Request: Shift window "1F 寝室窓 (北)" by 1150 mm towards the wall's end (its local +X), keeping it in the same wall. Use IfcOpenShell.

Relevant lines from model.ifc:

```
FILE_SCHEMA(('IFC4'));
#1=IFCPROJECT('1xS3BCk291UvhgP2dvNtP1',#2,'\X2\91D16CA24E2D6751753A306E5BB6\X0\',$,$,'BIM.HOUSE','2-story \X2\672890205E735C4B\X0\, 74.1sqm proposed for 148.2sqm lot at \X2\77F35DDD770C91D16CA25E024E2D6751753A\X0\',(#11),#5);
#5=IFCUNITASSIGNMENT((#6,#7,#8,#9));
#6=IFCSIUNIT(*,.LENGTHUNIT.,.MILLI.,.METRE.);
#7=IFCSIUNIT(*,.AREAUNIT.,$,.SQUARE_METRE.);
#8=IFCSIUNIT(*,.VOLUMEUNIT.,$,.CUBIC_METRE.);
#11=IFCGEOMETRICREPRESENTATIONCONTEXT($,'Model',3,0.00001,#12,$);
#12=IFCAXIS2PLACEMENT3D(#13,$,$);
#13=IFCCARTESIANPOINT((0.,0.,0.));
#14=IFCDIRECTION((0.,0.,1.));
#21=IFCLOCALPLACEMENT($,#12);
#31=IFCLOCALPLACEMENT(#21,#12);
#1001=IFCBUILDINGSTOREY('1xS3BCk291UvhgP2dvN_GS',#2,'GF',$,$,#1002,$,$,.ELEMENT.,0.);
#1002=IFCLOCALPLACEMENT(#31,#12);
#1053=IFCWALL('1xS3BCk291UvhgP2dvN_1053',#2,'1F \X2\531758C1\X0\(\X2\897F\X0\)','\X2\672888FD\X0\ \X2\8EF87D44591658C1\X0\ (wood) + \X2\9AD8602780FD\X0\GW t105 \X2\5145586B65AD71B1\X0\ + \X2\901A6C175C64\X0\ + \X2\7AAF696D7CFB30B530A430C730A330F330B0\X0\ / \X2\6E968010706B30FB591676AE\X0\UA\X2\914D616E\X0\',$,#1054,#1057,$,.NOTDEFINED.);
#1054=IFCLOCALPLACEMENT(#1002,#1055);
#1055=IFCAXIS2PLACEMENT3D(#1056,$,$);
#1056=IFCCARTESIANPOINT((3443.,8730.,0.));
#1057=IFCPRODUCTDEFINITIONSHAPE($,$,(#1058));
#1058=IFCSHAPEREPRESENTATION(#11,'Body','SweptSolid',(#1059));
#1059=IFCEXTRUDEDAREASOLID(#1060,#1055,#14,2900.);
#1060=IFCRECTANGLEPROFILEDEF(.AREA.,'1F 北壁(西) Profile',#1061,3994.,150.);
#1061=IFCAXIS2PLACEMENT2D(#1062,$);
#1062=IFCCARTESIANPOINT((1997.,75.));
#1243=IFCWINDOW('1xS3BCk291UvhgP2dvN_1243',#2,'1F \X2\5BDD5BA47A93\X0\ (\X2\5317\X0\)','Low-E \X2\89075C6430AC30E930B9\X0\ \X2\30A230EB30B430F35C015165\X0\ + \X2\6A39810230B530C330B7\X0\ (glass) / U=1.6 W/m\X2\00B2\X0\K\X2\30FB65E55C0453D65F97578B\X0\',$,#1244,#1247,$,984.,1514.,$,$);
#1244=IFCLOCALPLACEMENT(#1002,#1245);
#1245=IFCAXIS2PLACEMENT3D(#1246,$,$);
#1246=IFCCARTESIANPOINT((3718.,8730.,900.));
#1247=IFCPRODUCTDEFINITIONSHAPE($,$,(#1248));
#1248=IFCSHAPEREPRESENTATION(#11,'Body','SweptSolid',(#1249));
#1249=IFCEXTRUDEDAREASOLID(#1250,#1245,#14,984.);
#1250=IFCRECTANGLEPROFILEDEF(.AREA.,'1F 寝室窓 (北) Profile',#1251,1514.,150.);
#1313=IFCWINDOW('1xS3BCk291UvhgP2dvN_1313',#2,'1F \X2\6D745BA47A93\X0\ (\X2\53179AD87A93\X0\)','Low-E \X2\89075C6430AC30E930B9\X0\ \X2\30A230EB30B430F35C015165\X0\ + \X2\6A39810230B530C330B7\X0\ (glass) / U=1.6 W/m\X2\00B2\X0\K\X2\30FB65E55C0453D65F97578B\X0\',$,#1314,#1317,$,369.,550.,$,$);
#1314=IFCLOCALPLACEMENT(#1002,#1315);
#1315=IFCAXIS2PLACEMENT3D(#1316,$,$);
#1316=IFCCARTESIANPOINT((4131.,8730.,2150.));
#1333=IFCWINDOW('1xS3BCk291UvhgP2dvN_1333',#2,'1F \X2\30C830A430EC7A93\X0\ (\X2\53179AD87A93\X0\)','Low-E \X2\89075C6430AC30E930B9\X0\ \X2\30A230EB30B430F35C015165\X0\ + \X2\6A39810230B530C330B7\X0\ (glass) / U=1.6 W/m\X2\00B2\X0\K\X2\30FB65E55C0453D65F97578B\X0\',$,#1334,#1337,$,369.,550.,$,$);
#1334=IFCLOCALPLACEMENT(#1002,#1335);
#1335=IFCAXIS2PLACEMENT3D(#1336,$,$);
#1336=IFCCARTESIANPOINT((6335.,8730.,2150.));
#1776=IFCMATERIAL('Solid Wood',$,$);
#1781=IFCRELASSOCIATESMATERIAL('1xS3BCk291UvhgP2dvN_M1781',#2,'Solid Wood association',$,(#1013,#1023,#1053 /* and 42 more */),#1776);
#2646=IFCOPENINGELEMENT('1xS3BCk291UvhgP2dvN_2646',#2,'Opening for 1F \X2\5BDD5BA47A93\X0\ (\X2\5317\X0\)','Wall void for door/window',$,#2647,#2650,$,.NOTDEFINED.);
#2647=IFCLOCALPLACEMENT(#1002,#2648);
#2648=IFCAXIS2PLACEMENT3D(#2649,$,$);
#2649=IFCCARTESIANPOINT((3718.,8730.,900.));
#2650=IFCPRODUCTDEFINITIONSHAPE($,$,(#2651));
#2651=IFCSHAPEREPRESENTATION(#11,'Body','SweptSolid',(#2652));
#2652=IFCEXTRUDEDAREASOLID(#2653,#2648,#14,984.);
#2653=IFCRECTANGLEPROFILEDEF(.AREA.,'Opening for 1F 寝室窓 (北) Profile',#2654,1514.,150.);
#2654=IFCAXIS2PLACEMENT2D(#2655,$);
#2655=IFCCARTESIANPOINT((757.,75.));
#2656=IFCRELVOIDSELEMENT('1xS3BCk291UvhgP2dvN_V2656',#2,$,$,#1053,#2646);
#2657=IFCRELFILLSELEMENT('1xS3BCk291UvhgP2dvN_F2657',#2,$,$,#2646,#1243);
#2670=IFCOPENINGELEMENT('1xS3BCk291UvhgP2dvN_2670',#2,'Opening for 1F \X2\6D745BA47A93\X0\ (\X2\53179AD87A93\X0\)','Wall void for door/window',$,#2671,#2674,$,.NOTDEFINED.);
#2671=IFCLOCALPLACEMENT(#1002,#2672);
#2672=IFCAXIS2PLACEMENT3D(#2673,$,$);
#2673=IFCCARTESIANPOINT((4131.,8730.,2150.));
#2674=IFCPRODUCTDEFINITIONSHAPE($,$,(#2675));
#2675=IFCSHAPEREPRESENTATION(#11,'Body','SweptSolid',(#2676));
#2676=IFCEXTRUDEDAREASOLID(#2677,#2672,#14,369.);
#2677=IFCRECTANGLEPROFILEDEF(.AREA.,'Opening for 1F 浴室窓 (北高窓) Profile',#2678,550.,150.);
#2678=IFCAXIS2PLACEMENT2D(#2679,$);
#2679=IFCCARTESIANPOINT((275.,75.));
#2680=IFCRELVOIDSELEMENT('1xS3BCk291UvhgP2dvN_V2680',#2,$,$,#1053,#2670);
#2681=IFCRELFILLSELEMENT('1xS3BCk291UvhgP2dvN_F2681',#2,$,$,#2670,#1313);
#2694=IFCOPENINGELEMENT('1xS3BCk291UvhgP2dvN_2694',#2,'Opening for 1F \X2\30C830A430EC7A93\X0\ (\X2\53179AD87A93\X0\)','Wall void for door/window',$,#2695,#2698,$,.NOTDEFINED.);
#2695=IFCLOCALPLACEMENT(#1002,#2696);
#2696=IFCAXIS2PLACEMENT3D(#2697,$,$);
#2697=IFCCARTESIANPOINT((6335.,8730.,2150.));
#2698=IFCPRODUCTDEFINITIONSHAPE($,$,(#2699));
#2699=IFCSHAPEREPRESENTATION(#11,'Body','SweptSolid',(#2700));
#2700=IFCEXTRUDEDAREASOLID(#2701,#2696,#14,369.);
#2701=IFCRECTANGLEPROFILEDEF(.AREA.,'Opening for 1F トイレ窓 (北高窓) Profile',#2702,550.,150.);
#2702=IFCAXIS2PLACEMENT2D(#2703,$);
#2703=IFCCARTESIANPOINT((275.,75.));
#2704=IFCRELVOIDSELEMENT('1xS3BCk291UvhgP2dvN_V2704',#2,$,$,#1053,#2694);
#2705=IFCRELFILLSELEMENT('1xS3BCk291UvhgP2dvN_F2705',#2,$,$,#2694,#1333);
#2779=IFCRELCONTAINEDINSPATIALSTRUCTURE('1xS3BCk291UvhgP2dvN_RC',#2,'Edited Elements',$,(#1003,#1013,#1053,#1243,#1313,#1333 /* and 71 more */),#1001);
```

```python
import ifcopenshell
import ifcopenshell.api.geometry
import ifcopenshell.util.placement
import ifcopenshell.util.unit

model = ifcopenshell.open("model.ifc")
unit_scale = ifcopenshell.util.unit.calculate_unit_scale(model)

window = model.by_guid("1xS3BCk291UvhgP2dvN_1243")
opening = window.FillsVoids[0].RelatingOpeningElement
wall = opening.VoidsElements[0].RelatingBuildingElement

wall_matrix = ifcopenshell.util.placement.get_local_placement(wall.ObjectPlacement)
shift = wall_matrix[:3, 0] * 1.15 / unit_scale
before = ifcopenshell.util.placement.get_local_placement(window.ObjectPlacement)[:3, 3].copy()

# The window is not placed relative to its opening, so move both.
for product in (opening, window):
    matrix = ifcopenshell.util.placement.get_local_placement(product.ObjectPlacement)
    matrix[:3, 3] += shift
    ifcopenshell.api.geometry.edit_object_placement(model, product=product, matrix=matrix, is_si=False)

after = ifcopenshell.util.placement.get_local_placement(window.ObjectPlacement)[:3, 3]
print("window moved by", (after - before).round(3) + 0.0)

model.write("model_rev.ifc")
```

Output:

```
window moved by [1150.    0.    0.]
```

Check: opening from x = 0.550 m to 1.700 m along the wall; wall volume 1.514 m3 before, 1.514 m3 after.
